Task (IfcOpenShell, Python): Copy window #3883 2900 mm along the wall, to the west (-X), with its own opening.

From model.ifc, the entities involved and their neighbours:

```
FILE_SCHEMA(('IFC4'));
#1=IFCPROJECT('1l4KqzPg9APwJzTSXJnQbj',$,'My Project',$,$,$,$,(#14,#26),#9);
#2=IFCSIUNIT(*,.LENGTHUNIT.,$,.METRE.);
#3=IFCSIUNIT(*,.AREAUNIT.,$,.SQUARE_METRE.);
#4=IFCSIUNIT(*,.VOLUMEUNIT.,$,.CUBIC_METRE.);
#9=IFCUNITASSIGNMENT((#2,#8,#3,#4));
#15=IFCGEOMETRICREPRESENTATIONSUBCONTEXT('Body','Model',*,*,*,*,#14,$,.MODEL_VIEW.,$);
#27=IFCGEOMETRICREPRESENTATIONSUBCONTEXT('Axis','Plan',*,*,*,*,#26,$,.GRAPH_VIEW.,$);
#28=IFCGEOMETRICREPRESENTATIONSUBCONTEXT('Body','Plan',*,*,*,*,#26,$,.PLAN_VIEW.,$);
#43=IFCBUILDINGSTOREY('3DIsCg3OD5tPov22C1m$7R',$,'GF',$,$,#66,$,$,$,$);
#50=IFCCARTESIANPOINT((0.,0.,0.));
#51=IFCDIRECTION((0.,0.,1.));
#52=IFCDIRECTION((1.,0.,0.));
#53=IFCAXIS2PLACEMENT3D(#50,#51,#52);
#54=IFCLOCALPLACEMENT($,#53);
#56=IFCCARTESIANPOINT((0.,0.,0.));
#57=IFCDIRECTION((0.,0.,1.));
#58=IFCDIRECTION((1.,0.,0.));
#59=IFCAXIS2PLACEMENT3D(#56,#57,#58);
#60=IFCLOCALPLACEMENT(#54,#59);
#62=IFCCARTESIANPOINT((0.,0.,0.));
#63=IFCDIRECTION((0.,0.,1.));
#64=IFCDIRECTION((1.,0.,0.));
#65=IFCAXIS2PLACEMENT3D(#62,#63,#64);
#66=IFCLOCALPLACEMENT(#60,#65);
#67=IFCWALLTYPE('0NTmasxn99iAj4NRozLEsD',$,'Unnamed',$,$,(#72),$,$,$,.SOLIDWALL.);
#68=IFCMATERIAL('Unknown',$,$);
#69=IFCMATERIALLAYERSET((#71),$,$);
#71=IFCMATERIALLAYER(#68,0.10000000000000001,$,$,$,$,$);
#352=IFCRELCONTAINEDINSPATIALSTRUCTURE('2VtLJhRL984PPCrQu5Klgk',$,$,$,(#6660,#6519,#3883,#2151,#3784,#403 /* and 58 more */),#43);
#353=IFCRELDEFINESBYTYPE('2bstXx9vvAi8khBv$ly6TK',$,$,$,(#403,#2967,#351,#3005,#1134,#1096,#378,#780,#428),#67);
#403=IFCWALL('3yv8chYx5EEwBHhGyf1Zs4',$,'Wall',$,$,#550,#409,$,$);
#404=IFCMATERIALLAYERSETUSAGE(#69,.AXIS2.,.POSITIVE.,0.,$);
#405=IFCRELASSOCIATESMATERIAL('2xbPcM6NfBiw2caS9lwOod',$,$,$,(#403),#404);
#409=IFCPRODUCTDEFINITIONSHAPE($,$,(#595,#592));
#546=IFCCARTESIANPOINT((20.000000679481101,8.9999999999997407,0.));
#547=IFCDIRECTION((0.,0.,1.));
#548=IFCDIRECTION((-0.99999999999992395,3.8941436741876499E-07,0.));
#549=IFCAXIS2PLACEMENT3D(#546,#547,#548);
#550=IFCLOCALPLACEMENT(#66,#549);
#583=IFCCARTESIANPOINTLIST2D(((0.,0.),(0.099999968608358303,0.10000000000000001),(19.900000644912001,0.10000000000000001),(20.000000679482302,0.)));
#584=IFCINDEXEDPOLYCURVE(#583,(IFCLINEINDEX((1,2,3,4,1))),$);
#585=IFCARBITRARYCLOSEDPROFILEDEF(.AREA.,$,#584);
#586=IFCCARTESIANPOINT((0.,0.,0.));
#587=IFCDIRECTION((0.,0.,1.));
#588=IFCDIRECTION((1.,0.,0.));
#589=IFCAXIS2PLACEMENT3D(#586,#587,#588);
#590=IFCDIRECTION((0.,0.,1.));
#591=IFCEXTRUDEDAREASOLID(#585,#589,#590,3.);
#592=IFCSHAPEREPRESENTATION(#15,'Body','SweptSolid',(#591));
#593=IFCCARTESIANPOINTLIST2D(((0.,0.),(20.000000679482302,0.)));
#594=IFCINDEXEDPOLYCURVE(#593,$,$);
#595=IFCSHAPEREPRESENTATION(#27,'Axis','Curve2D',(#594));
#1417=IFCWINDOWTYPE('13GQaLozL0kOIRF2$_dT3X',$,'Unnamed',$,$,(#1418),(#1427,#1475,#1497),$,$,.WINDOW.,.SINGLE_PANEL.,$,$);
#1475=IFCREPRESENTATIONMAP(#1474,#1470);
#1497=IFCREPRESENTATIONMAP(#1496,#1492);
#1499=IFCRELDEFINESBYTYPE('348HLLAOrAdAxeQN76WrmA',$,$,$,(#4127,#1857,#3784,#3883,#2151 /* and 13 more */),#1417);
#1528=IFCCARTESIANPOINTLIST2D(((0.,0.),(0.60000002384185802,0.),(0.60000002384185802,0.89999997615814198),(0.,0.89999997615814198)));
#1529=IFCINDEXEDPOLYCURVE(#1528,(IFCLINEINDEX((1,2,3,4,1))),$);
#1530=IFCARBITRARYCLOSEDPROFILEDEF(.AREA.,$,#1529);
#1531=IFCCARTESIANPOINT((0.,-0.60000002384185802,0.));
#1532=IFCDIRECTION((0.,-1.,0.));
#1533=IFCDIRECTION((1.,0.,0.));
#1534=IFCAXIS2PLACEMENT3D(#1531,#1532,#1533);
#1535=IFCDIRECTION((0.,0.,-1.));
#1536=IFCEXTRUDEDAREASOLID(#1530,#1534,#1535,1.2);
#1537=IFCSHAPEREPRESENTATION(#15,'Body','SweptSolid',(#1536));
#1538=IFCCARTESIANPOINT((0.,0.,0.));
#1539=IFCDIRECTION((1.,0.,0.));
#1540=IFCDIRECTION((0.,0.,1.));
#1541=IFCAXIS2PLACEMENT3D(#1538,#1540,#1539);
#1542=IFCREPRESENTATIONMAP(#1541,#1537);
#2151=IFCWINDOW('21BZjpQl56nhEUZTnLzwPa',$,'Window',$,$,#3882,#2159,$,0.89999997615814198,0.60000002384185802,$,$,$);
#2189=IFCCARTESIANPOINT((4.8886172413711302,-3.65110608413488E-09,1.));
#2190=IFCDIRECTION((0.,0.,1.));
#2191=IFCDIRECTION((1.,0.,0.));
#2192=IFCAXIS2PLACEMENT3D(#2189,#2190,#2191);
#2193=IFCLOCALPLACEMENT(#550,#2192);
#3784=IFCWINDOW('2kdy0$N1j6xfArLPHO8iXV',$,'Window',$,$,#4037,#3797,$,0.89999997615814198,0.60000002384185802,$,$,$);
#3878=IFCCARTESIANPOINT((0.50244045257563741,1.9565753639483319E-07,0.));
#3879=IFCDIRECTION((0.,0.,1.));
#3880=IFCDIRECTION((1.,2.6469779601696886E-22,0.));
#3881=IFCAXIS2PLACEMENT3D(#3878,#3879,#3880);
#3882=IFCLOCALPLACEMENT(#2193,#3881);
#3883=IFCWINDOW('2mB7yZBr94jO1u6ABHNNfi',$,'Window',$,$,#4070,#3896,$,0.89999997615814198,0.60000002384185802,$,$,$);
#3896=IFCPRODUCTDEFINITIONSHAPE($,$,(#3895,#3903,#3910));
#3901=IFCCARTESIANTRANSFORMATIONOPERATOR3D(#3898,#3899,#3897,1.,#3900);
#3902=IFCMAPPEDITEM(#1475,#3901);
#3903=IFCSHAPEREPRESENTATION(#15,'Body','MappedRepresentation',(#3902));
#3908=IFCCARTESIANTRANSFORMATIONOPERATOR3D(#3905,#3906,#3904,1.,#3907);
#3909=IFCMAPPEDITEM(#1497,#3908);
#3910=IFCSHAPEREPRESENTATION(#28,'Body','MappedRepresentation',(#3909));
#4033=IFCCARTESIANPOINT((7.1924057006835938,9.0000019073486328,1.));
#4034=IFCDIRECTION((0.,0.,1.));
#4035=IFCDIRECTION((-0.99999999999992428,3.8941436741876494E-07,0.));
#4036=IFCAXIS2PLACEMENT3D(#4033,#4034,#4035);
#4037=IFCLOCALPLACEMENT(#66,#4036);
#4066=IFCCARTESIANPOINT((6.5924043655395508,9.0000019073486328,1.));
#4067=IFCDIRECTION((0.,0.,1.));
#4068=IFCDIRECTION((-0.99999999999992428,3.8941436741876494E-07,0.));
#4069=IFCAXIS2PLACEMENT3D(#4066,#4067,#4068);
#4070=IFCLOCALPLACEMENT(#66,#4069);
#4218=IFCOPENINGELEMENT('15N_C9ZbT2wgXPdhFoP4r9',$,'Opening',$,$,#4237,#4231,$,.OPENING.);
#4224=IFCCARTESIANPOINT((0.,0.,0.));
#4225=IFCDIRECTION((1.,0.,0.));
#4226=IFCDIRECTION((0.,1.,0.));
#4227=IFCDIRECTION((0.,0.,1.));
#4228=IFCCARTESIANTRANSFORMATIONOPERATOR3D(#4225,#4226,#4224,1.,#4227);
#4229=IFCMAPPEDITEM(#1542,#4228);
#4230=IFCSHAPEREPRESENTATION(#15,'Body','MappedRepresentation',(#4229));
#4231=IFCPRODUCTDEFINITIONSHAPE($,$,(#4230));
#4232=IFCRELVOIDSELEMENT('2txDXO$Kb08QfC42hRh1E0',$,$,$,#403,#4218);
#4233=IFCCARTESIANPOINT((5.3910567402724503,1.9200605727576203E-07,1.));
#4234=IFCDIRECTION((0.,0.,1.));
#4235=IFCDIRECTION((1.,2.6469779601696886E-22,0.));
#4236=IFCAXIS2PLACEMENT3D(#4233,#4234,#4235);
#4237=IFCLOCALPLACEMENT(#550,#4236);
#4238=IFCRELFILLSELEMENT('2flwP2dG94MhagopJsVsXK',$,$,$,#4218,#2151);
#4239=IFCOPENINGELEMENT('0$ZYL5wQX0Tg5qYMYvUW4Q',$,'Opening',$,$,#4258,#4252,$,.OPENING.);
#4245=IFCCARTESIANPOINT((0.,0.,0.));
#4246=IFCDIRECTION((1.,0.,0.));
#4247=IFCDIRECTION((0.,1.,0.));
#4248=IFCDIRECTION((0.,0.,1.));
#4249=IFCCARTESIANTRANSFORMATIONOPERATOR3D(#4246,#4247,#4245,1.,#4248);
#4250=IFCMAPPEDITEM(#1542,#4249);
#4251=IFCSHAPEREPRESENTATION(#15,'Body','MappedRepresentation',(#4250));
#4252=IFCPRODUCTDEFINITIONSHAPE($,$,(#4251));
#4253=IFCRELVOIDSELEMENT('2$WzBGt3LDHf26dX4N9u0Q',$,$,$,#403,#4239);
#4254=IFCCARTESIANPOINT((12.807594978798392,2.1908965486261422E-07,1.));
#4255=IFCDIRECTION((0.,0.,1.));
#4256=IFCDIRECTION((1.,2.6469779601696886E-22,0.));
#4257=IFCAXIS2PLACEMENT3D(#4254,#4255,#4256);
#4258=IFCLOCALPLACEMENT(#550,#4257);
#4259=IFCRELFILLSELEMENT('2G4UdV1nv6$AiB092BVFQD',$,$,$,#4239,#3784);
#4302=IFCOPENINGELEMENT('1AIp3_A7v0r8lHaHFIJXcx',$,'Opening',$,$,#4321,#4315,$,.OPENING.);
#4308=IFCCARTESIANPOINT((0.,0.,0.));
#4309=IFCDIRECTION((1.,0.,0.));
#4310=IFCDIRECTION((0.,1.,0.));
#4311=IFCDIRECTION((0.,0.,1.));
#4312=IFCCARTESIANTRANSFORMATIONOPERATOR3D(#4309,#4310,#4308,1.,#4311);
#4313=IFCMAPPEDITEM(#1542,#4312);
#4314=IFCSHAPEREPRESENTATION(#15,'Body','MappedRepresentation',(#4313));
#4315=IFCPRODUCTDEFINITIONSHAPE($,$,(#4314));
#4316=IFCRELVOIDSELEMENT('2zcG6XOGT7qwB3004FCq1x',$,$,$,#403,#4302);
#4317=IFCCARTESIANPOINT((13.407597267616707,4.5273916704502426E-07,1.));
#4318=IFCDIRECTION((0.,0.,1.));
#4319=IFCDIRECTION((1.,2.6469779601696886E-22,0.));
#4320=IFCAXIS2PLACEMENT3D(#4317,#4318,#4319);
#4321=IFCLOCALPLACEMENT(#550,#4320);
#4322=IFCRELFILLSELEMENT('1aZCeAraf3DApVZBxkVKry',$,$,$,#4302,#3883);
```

```python
import ifcopenshell
import ifcopenshell.api.feature
import ifcopenshell.api.geometry
import ifcopenshell.api.root
import ifcopenshell.geom
import ifcopenshell.util.element
import ifcopenshell.util.placement
import ifcopenshell.util.shape
import ifcopenshell.util.unit

model = ifcopenshell.open("model.ifc")
unit_scale = ifcopenshell.util.unit.calculate_unit_scale(model)
settings = ifcopenshell.geom.settings()


def volume(element):
    """Net volume in cubic metres, openings subtracted."""
    shape = ifcopenshell.geom.create_shape(settings, element)
    return ifcopenshell.util.shape.get_volume(shape.geometry)


window = model.by_id(3883)
opening = window.FillsVoids[0].RelatingOpeningElement
wall = opening.VoidsElements[0].RelatingBuildingElement
before = volume(wall)
shift = ifcopenshell.util.placement.get_local_placement(wall.ObjectPlacement)[:3, 0] * 2.9 / unit_scale

# copy_class copies the void relationship, type, container and properties, but no geometry.
new_opening = ifcopenshell.api.root.copy_class(model, product=opening)
new_opening.Representation = ifcopenshell.util.element.copy_deep(
    model, opening.Representation, exclude=["IfcGeometricRepresentationContext", "IfcRepresentationMap"]
)
new_window = ifcopenshell.api.root.copy_class(model, product=window)
new_window.Representation = ifcopenshell.util.element.copy_deep(
    model, window.Representation, exclude=["IfcGeometricRepresentationContext", "IfcRepresentationMap"]
)
ifcopenshell.api.feature.add_filling(model, opening=new_opening, element=new_window)

for old, new in ((opening, new_opening), (window, new_window)):
    matrix = ifcopenshell.util.placement.get_local_placement(old.ObjectPlacement)
    matrix[:3, 3] += shift
    ifcopenshell.api.geometry.edit_object_placement(model, product=new, matrix=matrix, is_si=False)

after = volume(wall)

print(f"wall volume {before:.3f} -> {after:.3f} m3")

model.write("model_v2.ifc")
```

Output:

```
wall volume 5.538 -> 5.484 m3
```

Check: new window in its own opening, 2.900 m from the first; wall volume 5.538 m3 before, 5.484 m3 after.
